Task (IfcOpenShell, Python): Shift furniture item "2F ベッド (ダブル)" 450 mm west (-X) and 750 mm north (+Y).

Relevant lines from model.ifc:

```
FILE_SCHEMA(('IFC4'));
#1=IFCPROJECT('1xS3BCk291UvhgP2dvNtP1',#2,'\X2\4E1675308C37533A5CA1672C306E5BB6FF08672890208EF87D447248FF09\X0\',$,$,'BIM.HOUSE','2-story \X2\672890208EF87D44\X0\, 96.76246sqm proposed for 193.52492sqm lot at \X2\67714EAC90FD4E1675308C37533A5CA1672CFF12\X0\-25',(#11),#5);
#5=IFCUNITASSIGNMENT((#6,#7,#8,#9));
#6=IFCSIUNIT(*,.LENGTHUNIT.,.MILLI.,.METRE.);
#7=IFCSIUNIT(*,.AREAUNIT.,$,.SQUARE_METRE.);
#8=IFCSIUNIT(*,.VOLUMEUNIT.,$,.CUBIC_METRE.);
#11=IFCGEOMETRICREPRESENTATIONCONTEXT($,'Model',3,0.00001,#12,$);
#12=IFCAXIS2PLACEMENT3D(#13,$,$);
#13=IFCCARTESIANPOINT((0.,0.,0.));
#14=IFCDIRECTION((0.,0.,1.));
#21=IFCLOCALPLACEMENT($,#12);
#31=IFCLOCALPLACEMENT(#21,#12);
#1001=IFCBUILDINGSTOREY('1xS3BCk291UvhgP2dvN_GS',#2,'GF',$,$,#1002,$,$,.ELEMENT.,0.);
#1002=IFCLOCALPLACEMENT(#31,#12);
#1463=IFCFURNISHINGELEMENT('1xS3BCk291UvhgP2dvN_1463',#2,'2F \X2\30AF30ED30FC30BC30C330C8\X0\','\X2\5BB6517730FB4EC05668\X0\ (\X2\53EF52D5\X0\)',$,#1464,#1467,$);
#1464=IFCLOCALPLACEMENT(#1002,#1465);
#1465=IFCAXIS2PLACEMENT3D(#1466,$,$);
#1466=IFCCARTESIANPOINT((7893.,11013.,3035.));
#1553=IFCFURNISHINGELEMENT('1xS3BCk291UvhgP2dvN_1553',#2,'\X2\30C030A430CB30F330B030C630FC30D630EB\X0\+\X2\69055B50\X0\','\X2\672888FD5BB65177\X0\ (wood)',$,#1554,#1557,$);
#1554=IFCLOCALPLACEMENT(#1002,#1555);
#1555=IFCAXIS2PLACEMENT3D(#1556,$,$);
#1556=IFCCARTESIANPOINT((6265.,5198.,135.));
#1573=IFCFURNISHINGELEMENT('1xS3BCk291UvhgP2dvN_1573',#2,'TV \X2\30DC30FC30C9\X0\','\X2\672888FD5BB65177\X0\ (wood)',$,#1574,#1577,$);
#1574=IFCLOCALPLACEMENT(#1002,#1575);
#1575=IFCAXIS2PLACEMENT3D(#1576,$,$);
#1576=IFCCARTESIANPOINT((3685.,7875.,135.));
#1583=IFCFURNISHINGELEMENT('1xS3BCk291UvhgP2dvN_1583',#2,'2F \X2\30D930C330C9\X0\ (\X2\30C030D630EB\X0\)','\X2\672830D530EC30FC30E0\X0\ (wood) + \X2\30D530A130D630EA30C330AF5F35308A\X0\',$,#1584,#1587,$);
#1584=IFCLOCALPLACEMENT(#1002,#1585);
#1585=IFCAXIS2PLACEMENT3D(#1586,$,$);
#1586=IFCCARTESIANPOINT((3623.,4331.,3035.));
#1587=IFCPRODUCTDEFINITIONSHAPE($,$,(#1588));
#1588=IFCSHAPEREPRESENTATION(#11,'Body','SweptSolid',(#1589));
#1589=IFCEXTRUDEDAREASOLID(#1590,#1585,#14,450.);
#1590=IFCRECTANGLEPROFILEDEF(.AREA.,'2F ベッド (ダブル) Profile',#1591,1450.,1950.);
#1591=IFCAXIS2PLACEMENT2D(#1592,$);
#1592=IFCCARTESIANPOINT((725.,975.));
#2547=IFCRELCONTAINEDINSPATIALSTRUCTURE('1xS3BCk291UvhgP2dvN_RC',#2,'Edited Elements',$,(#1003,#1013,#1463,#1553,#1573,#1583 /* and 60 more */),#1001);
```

```python
import ifcopenshell
import ifcopenshell.api.geometry
import ifcopenshell.util.placement
import ifcopenshell.util.unit

model = ifcopenshell.open("model.ifc")
unit_scale = ifcopenshell.util.unit.calculate_unit_scale(model)

item = model.by_guid("1xS3BCk291UvhgP2dvN_1583")
matrix = ifcopenshell.util.placement.get_local_placement(item.ObjectPlacement)
matrix[0, 3] -= 0.45 / unit_scale
matrix[1, 3] += 0.75 / unit_scale
ifcopenshell.api.geometry.edit_object_placement(model, product=item, matrix=matrix, is_si=False)

print(ifcopenshell.util.placement.get_local_placement(item.ObjectPlacement).round(3) + 0.0)

model.write("model_rev.ifc")
```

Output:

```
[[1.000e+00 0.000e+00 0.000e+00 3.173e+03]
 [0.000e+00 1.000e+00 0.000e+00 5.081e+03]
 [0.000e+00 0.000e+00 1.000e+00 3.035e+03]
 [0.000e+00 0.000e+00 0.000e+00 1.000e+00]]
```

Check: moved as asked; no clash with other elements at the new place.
